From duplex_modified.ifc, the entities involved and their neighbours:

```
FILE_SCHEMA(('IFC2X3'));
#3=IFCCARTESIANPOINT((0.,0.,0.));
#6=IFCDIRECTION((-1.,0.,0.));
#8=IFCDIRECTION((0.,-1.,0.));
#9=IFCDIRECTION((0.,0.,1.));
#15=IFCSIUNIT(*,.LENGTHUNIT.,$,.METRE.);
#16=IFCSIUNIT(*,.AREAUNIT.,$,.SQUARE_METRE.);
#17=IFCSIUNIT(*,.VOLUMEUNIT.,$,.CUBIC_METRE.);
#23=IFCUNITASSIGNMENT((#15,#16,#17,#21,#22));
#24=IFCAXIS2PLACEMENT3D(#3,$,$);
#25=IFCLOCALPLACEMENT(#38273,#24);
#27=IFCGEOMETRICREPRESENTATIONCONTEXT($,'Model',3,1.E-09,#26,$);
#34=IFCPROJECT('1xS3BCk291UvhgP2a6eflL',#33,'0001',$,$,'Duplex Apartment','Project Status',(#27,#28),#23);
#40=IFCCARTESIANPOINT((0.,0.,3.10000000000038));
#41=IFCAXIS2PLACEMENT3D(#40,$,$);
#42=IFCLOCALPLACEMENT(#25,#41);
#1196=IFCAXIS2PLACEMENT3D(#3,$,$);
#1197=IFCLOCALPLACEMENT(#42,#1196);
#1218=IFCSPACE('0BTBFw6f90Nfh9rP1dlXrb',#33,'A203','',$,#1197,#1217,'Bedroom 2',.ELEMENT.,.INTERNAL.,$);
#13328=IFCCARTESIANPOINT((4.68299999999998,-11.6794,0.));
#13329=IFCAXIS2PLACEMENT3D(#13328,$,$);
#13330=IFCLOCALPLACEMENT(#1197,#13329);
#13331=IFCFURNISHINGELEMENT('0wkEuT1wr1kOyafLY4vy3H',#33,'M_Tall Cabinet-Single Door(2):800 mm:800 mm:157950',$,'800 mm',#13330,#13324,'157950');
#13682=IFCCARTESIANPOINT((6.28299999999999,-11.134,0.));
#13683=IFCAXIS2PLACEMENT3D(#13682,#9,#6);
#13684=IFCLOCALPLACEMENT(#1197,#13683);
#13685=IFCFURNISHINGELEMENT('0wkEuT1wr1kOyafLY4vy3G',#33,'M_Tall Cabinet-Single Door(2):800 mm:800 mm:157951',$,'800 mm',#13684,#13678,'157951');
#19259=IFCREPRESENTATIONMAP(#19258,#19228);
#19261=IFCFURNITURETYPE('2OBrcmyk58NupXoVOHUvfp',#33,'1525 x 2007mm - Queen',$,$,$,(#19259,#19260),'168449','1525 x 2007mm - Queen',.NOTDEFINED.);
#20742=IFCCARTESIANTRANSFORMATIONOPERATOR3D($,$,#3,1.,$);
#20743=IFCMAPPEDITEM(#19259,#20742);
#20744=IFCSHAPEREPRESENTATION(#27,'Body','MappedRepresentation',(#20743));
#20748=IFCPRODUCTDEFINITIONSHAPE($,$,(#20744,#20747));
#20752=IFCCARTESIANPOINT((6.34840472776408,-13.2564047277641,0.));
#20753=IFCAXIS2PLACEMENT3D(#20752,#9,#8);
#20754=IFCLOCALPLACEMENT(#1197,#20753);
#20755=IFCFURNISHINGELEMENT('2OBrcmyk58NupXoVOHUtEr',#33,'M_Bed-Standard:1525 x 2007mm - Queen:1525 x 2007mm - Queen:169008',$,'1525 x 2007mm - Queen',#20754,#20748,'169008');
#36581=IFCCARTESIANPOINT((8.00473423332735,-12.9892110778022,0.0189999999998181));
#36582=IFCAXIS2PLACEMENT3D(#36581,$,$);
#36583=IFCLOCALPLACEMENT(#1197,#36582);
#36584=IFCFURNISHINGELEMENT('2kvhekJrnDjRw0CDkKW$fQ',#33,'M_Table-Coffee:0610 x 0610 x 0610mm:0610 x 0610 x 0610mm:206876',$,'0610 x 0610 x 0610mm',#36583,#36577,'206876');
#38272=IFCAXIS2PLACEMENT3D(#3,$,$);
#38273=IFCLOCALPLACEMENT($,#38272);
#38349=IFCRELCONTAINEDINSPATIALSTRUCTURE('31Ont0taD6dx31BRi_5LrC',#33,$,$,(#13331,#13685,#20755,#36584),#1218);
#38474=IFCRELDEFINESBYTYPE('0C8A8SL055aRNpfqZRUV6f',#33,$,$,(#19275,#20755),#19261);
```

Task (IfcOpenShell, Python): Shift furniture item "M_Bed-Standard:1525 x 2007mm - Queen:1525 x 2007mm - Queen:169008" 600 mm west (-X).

```python
import ifcopenshell
import ifcopenshell.api.geometry
import ifcopenshell.util.placement
import ifcopenshell.util.unit

model = ifcopenshell.open("duplex_modified.ifc")
unit_scale = ifcopenshell.util.unit.calculate_unit_scale(model)

item = model.by_id(20755)
matrix = ifcopenshell.util.placement.get_local_placement(item.ObjectPlacement)
matrix[0, 3] -= 0.6 / unit_scale
ifcopenshell.api.geometry.edit_object_placement(model, product=item, matrix=matrix, is_si=False)

print(ifcopenshell.util.placement.get_local_placement(item.ObjectPlacement).round(3) + 0.0)

model.write("duplex_modified_edited.ifc")
```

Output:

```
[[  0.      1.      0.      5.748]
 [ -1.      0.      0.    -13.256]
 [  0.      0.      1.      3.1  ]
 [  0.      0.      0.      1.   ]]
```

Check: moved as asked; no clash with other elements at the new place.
